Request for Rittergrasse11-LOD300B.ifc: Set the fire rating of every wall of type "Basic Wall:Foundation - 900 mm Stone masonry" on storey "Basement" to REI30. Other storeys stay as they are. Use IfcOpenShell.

First a look at what the model holds.

```python
import ifcopenshell
import ifcopenshell.util.element

model = ifcopenshell.open("Rittergrasse11-LOD300B.ifc")
print(model.schema)
storey = next(s for s in model.by_type("IfcBuildingStorey") if s.Name == "Basement")
walls = [e for e in ifcopenshell.util.element.get_decomposition(storey) if e.is_a("IfcWall")]
seen = {}
for e in walls:
    element_type = ifcopenshell.util.element.get_type(e)
    key = (element_type.Name if element_type != e and element_type else None, ifcopenshell.util.element.get_pset(e, "Pset_WallCommon", "FireRating"))
    seen[key] = seen.get(key, 0) + 1
for (name, value), count in sorted(seen.items(), key=str):
    print(count, "x", name, "|", value)
```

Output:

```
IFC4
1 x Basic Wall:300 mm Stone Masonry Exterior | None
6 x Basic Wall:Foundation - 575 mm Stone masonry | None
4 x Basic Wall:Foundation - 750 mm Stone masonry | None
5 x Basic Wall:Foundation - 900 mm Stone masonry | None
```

```python
import ifcopenshell
import ifcopenshell.api.pset
import ifcopenshell.util.element

model = ifcopenshell.open("Rittergrasse11-LOD300B.ifc")

storey = next(s for s in model.by_type("IfcBuildingStorey") if s.Name == "Basement")
walls = [e for e in ifcopenshell.util.element.get_decomposition(storey) if e.is_a("IfcWall")]

count = 0
for e in walls:
    element_type = ifcopenshell.util.element.get_type(e)
    if element_type in (None, e) or element_type.Name != "Basic Wall:Foundation - 900 mm Stone masonry":
        continue
    # add_pset returns the element's existing set when there is one.
    pset = ifcopenshell.api.pset.add_pset(model, product=e, name="Pset_WallCommon")
    ifcopenshell.api.pset.edit_pset(model, pset=pset, properties={"FireRating": "REI30"})
    count += 1

print(count, "walls updated")

model.write("Rittergrasse11-LOD300B_rev.ifc")
```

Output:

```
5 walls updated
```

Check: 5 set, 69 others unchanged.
